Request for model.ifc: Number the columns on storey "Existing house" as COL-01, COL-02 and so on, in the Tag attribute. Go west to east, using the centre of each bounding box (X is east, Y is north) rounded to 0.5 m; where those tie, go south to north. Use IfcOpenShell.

First a look at what the model holds.

```python
import ifcopenshell
import ifcopenshell.util.element
import ifcopenshell.util.placement

model = ifcopenshell.open("model.ifc")
print(model.schema)
storey = next(s for s in model.by_type("IfcBuildingStorey") if s.Name == "Existing house")
columns = [e for e in ifcopenshell.util.element.get_decomposition(storey) if e.is_a("IfcColumn")]
for e in sorted(columns, key=lambda e: e.id()):
    origin = ifcopenshell.util.placement.get_local_placement(e.ObjectPlacement)[:3, 3]
    print(e.id(), e.Tag, e.Name, origin.round(2) + 0.0, sep=" | ")
```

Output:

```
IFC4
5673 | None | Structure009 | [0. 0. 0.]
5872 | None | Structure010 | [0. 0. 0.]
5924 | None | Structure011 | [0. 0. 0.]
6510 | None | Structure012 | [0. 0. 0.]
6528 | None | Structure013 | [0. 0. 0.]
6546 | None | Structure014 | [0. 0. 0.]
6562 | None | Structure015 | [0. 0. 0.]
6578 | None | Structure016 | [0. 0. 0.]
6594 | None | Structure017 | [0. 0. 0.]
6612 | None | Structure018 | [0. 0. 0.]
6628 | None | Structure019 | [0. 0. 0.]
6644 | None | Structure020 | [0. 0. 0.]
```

```python
import ifcopenshell
import ifcopenshell.geom
import ifcopenshell.util.element
import ifcopenshell.util.shape

model = ifcopenshell.open("model.ifc")
settings = ifcopenshell.geom.settings()
settings.set("use-world-coords", True)


def centre(element):
    shape = ifcopenshell.geom.create_shape(settings, element)
    return ifcopenshell.util.shape.get_bbox_centroid(shape.geometry)


storey = next(s for s in model.by_type("IfcBuildingStorey") if s.Name == "Existing house")
columns = [e for e in ifcopenshell.util.element.get_decomposition(storey) if e.is_a("IfcColumn")]

# Insertion points can sit at a corner or the storey origin, so sort by the geometry (in metres).
centres = {e: centre(e) for e in columns}
columns.sort(key=lambda e: (round(centres[e][0] / 0.5), centres[e][1]))

for i, e in enumerate(columns, start=1):
    number = f"COL-{i:02d}"
    e.Tag = number
    print(e.id(), number)

model.write("model_updated.ifc")
```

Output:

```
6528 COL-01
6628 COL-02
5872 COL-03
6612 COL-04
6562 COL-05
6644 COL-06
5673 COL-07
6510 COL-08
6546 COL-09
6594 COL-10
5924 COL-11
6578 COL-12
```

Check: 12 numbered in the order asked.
